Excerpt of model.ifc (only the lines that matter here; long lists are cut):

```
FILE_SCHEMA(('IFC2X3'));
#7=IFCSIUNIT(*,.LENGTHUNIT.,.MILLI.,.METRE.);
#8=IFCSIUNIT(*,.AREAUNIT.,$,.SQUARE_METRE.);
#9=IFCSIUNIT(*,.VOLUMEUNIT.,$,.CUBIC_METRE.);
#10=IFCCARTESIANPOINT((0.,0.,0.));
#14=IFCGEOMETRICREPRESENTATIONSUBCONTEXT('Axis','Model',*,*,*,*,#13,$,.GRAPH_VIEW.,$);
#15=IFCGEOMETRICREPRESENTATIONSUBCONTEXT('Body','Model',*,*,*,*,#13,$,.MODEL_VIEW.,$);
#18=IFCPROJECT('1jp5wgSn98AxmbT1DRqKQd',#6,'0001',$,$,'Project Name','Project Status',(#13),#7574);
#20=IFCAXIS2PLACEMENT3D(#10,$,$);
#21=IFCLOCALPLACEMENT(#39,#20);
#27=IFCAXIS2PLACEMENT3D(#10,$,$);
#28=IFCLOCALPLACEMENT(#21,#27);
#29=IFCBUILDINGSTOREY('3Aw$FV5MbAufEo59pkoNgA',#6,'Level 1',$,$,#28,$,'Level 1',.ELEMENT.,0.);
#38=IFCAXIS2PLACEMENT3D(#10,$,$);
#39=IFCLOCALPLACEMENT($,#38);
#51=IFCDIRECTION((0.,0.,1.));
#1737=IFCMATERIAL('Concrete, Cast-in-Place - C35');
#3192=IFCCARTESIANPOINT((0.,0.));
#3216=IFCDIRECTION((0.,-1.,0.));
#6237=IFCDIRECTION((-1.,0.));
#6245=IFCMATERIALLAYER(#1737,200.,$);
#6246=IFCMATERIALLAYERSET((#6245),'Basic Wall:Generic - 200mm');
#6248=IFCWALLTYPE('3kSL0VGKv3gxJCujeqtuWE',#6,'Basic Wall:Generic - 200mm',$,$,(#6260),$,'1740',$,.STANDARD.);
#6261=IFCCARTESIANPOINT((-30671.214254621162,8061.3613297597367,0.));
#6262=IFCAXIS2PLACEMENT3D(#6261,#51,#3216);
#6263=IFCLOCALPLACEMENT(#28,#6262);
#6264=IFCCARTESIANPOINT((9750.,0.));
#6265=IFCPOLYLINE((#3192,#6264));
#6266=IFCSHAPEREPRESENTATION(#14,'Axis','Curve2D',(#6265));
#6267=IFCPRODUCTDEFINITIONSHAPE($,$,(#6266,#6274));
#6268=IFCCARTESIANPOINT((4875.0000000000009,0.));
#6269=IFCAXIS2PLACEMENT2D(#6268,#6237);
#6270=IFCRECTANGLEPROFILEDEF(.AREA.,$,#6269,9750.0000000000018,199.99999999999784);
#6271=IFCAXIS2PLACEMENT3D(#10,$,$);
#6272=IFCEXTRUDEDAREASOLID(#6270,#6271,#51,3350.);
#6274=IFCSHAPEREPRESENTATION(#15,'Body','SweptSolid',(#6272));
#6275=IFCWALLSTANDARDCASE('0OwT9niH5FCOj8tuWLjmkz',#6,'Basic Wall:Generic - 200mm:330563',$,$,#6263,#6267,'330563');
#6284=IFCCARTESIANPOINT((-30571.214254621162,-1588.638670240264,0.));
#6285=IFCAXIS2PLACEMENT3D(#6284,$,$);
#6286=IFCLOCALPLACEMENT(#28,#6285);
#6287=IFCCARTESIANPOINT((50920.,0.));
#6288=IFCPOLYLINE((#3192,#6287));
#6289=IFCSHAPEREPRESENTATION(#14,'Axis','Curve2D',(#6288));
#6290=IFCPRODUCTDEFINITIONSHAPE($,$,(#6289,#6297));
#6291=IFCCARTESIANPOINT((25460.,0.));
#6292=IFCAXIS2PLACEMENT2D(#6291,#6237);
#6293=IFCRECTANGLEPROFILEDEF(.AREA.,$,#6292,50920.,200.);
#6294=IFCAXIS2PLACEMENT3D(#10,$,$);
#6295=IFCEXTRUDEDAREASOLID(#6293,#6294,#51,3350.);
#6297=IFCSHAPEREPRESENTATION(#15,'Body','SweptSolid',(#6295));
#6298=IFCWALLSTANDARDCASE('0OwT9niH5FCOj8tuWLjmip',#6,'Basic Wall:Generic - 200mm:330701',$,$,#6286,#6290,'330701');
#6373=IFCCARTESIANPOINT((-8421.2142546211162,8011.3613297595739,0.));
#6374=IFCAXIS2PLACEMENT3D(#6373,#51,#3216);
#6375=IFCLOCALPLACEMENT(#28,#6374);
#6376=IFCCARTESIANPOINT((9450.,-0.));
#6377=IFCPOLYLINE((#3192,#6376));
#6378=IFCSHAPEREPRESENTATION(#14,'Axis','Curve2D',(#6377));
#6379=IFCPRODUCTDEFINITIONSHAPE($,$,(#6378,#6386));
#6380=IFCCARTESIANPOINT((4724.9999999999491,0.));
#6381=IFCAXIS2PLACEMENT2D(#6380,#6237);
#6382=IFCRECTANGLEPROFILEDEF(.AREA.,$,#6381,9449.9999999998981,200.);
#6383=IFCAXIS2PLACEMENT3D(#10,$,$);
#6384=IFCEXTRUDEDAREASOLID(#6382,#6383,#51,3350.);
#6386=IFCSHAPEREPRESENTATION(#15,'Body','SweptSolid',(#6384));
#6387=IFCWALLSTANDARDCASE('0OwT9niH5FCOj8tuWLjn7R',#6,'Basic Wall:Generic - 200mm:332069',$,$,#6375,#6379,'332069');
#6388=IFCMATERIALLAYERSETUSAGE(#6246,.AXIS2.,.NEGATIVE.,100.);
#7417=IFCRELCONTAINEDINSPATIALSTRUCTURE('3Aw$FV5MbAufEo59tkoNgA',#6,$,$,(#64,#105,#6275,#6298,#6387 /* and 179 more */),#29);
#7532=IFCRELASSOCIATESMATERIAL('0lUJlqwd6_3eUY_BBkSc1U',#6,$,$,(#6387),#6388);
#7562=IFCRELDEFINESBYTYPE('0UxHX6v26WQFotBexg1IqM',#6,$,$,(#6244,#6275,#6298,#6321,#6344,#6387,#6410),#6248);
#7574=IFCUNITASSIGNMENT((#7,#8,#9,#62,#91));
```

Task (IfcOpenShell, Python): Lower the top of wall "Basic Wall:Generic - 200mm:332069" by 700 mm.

```python
import ifcopenshell
import ifcopenshell.geom
import ifcopenshell.util.representation
import ifcopenshell.util.shape

model = ifcopenshell.open("model.ifc")
settings = ifcopenshell.geom.settings()


def volume(element):
    """Net volume in cubic metres, openings subtracted."""
    shape = ifcopenshell.geom.create_shape(settings, element)
    return ifcopenshell.util.shape.get_volume(shape.geometry)


wall = model.by_guid("0OwT9niH5FCOj8tuWLjn7R")
before = volume(wall)

body = ifcopenshell.util.representation.get_representation(wall, "Model", "Body")
solid = body.Items[0]
old_height = solid.Depth
solid.Depth -= 700.0
after = volume(wall)

print(f"height {old_height:g} -> {solid.Depth:g}, volume {before:.3f} -> {after:.3f} m3")

model.write("model-out.ifc")
```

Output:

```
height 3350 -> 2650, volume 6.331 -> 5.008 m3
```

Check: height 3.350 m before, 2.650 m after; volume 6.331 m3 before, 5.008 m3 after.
